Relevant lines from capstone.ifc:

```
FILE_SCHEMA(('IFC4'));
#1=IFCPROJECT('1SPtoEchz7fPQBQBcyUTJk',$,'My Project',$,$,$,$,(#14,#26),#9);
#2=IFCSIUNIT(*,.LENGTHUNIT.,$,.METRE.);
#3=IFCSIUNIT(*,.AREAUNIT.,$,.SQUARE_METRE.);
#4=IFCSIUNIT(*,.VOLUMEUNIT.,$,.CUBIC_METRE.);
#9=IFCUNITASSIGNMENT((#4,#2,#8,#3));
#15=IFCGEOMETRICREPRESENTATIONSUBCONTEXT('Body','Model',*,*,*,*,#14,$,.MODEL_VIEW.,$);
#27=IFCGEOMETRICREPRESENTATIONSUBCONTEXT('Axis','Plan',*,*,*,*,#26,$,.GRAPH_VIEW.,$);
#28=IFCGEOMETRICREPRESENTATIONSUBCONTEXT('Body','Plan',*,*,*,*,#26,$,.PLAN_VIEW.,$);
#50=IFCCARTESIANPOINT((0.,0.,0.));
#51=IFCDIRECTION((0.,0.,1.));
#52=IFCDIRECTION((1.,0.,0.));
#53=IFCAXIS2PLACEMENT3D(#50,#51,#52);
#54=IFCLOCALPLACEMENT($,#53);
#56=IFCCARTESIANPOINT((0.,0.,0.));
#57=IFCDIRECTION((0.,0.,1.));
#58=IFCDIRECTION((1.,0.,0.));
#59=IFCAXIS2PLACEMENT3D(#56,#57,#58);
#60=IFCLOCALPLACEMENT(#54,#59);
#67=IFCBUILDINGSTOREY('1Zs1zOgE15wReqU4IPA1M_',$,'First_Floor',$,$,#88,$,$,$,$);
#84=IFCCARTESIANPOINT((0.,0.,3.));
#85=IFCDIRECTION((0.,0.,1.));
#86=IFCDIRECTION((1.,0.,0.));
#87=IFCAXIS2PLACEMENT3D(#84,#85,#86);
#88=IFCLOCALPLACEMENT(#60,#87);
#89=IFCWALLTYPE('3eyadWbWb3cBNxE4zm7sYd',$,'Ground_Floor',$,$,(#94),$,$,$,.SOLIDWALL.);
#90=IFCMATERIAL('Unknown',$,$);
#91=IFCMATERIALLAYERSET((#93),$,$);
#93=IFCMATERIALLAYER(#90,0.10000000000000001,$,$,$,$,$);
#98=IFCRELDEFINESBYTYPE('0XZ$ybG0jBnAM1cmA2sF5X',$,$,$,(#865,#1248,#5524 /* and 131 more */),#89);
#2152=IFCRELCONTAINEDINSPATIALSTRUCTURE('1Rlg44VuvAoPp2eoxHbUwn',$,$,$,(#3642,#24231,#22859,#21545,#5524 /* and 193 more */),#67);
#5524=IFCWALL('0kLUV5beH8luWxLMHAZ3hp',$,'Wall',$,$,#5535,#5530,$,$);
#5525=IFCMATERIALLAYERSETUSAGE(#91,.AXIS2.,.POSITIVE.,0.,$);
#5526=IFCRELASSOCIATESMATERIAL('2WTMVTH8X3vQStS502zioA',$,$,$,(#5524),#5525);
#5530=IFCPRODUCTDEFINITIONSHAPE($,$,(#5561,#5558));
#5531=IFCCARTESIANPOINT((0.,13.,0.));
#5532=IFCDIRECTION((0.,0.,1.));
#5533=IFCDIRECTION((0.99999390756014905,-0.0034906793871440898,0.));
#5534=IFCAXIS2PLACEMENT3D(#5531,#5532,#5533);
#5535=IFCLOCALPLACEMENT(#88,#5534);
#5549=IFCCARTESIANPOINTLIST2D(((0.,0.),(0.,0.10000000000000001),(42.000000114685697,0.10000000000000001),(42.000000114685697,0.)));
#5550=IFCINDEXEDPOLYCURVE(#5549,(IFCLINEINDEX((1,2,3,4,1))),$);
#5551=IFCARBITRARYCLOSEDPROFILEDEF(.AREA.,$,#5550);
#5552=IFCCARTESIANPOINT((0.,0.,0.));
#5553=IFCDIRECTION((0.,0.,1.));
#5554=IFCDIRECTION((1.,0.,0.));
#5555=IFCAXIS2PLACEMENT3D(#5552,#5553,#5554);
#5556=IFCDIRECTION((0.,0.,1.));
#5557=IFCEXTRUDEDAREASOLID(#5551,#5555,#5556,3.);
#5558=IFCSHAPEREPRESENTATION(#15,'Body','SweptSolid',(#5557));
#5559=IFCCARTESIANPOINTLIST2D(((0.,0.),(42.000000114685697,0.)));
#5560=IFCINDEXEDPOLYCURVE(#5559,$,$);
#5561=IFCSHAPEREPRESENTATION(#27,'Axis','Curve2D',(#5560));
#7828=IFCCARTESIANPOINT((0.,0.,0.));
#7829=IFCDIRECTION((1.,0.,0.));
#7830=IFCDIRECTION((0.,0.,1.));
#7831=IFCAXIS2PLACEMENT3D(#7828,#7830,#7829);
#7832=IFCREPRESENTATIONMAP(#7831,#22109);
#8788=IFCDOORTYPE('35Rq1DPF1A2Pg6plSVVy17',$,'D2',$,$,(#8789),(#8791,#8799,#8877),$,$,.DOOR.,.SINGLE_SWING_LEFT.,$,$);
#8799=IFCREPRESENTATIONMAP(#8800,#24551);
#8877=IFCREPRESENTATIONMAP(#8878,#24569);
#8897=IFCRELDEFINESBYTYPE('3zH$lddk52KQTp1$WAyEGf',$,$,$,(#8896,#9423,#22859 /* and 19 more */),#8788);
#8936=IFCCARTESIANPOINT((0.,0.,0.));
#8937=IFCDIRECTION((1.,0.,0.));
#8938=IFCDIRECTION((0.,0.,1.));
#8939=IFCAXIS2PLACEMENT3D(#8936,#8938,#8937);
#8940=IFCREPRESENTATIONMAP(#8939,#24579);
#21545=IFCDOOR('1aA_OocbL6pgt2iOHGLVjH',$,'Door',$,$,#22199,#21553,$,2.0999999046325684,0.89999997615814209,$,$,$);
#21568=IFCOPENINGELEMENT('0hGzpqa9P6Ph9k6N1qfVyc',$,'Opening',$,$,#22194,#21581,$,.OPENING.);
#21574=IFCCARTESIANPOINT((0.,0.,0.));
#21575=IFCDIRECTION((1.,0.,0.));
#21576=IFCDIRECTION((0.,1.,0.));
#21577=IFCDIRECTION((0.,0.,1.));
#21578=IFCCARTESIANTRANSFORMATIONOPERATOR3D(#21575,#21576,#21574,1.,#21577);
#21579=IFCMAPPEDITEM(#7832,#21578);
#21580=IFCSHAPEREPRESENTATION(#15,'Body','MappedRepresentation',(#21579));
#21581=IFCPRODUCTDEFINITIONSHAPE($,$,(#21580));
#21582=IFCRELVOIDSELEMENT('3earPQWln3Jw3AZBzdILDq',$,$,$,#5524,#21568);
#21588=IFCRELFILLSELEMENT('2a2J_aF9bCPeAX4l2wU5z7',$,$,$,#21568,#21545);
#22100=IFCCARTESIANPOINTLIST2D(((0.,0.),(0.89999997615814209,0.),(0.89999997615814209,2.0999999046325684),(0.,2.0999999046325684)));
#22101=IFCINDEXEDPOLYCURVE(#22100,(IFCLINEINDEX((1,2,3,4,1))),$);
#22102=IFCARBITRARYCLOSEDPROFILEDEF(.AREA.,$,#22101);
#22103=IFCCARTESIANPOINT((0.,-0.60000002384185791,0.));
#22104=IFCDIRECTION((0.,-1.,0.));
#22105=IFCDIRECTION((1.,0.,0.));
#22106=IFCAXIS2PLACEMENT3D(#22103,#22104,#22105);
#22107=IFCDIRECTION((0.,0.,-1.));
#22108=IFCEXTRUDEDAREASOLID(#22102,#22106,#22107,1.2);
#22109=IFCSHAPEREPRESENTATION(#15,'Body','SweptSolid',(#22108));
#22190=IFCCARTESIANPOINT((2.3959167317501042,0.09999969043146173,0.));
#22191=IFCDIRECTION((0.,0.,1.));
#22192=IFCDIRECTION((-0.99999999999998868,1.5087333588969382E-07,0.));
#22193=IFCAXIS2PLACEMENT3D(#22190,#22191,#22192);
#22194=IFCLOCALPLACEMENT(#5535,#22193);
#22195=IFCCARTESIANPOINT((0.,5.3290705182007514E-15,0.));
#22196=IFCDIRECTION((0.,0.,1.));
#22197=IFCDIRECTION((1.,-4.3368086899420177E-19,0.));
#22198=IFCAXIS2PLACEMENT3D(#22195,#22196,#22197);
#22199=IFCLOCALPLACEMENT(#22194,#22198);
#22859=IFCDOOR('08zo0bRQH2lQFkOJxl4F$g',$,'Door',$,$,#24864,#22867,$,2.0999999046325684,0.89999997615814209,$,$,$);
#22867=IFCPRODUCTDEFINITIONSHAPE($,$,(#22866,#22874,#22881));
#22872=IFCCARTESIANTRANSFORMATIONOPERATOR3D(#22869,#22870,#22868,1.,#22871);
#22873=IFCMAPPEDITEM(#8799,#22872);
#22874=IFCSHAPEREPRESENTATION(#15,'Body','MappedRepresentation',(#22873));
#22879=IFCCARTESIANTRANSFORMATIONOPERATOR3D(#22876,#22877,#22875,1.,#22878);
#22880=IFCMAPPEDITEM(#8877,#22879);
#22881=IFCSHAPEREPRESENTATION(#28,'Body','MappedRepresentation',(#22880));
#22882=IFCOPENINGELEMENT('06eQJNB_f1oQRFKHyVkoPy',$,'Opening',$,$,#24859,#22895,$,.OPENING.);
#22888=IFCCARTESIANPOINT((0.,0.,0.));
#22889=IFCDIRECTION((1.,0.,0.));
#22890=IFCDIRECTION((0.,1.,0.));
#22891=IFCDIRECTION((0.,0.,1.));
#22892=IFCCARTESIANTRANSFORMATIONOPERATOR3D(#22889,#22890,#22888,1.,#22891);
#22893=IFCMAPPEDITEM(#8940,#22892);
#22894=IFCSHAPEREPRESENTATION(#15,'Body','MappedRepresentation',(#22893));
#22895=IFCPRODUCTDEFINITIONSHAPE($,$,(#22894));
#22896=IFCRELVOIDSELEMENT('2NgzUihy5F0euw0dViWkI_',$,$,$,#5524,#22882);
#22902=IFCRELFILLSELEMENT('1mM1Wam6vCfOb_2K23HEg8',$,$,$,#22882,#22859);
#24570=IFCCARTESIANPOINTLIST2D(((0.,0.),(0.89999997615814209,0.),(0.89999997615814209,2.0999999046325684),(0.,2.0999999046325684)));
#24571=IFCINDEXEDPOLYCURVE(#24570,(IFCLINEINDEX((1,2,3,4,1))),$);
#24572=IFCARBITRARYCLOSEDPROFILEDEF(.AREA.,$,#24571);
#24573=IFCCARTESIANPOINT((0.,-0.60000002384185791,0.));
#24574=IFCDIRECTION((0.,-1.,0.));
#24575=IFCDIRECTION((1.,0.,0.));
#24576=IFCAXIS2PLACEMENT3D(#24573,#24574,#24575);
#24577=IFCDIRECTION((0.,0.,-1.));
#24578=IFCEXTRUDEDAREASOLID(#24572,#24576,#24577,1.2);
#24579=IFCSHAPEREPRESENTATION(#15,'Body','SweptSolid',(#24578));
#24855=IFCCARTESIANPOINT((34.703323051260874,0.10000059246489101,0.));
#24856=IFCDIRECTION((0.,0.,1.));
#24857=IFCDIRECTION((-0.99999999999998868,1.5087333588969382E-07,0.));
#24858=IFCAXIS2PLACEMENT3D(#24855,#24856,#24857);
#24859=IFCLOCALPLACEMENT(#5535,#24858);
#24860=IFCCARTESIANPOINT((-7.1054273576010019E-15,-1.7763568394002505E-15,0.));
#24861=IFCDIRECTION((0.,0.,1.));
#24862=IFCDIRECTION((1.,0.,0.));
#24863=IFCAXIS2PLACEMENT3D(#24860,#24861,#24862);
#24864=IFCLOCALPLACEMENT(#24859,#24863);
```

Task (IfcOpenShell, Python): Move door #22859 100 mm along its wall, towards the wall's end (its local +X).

```python
import ifcopenshell
import ifcopenshell.api.geometry
import ifcopenshell.util.placement

model = ifcopenshell.open("capstone.ifc")

door = model.by_id(22859)
opening = door.FillsVoids[0].RelatingOpeningElement
wall = opening.VoidsElements[0].RelatingBuildingElement

wall_matrix = ifcopenshell.util.placement.get_local_placement(wall.ObjectPlacement)
shift = wall_matrix[:3, 0] * 0.1
before = ifcopenshell.util.placement.get_local_placement(door.ObjectPlacement)[:3, 3].copy()

# The door is placed relative to its opening, so it follows when the opening moves.
matrix = ifcopenshell.util.placement.get_local_placement(opening.ObjectPlacement)
matrix[:3, 3] += shift
ifcopenshell.api.geometry.edit_object_placement(
    model, product=opening, matrix=matrix, is_si=False, should_transform_children=True
)

after = ifcopenshell.util.placement.get_local_placement(door.ObjectPlacement)[:3, 3]
print("door moved by", (after - before).round(3) + 0.0)

model.write("capstone_edited.ifc")
```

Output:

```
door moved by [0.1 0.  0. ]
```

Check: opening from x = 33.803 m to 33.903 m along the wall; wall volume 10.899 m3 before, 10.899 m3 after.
